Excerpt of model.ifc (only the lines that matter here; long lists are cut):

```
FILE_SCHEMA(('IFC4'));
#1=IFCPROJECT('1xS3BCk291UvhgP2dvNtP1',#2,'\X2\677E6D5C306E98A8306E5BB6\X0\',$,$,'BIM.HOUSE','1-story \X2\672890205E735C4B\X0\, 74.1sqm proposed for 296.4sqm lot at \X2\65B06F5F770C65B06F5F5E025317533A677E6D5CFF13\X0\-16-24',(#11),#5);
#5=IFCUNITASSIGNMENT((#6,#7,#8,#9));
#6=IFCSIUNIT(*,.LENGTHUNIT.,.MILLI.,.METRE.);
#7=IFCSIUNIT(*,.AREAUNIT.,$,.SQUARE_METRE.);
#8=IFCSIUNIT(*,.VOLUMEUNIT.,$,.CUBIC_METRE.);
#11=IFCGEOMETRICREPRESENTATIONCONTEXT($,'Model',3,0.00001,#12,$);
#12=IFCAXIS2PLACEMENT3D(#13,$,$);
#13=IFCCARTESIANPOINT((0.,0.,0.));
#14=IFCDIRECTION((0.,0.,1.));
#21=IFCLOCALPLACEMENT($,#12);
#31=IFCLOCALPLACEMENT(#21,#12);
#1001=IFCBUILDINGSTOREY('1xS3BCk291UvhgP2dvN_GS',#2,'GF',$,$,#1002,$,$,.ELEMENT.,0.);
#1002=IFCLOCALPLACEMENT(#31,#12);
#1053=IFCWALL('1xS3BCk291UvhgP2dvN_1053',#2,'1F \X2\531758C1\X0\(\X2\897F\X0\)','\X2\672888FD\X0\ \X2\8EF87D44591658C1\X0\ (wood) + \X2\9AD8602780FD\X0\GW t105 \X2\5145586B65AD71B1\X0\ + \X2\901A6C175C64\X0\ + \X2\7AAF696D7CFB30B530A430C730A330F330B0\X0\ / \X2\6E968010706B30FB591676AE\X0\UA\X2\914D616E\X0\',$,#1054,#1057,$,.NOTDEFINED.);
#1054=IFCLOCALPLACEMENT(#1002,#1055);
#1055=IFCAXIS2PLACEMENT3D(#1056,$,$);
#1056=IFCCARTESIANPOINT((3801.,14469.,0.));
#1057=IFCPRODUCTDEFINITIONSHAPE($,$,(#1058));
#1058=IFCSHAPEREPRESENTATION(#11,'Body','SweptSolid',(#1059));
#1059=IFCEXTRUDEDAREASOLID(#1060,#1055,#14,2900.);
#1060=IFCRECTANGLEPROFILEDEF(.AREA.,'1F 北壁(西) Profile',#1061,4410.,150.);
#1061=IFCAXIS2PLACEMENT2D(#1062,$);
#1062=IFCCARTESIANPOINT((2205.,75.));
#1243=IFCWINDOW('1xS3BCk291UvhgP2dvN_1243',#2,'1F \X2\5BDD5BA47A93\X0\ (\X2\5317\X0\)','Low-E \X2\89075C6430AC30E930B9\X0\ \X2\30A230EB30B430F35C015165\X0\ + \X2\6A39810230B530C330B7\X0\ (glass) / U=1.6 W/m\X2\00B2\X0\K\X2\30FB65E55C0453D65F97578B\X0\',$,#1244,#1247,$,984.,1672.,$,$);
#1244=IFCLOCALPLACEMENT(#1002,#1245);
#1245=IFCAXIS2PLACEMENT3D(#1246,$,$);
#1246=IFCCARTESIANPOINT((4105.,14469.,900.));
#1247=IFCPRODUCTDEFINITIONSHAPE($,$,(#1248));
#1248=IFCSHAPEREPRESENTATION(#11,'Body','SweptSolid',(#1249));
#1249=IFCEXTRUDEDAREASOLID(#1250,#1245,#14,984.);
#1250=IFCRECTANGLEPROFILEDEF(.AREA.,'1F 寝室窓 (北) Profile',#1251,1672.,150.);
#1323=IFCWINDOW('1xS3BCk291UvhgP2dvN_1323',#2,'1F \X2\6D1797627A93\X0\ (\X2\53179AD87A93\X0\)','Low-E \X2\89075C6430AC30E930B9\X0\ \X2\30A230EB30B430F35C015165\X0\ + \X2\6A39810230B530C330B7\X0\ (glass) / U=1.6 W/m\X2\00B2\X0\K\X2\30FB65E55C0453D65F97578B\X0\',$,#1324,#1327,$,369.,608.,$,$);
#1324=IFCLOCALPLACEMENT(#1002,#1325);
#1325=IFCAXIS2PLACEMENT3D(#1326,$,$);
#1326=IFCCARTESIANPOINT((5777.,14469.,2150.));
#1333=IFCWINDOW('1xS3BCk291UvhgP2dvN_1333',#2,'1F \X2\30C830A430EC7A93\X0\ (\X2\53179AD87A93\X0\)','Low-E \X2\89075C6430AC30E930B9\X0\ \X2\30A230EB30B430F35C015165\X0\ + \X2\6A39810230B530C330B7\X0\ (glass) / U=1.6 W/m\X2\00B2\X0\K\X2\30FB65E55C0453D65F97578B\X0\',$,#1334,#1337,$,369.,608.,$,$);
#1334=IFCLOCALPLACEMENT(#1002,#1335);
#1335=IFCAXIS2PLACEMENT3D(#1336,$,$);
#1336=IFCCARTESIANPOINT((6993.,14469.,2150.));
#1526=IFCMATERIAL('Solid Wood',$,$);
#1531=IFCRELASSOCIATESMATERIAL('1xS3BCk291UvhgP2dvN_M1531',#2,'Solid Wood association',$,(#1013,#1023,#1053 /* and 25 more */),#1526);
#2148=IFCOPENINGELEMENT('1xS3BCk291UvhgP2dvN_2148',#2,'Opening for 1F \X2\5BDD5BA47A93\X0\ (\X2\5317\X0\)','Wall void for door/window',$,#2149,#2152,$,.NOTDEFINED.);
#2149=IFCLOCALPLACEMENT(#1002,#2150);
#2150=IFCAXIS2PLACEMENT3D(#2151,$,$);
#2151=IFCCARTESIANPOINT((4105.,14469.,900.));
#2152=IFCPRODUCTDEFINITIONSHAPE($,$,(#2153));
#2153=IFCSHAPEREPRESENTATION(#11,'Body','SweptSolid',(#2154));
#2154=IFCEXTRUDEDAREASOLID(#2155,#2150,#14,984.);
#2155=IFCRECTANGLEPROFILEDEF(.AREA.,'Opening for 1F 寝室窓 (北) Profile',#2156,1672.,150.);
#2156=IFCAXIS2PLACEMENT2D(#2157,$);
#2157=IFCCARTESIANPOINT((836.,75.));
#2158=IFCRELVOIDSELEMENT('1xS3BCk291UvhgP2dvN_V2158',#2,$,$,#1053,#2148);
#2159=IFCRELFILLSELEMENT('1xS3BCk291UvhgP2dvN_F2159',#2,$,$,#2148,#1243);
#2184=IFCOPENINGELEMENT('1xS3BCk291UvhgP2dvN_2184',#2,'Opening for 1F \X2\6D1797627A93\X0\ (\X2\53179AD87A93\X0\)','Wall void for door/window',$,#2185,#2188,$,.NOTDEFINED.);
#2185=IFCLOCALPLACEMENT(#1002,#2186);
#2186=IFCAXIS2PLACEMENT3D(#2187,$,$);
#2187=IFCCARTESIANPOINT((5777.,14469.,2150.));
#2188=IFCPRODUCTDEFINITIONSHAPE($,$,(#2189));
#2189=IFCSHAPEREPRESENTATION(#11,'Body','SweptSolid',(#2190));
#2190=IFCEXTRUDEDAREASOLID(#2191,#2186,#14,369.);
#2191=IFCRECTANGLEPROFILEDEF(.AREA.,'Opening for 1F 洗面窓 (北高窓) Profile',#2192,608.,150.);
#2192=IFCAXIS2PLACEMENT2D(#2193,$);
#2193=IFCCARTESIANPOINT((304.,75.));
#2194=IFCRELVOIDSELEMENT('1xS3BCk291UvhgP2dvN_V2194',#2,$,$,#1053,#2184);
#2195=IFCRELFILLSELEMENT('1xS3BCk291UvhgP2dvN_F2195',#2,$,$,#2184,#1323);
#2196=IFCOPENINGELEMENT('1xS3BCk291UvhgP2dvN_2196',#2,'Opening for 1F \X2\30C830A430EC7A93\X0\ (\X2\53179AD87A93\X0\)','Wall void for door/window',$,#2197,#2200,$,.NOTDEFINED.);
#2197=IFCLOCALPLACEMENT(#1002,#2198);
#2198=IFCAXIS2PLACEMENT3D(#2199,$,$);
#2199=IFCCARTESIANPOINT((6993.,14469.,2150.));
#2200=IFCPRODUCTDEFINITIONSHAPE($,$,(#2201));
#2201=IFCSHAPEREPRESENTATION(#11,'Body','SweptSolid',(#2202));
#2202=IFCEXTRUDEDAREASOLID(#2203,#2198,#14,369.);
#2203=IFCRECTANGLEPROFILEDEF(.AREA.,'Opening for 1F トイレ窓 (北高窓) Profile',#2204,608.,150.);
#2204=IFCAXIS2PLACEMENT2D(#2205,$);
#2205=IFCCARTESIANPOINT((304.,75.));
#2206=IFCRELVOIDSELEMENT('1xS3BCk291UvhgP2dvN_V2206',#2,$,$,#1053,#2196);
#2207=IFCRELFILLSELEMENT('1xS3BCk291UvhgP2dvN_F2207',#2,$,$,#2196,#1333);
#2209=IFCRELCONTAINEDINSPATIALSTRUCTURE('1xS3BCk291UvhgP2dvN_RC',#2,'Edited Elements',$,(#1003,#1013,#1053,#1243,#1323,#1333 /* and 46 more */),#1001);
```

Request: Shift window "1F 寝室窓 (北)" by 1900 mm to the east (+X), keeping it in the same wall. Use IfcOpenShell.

```python
import ifcopenshell
import ifcopenshell.api.geometry
import ifcopenshell.util.placement
import ifcopenshell.util.unit

model = ifcopenshell.open("model.ifc")
unit_scale = ifcopenshell.util.unit.calculate_unit_scale(model)

window = model.by_id(1243)
opening = window.FillsVoids[0].RelatingOpeningElement
wall = opening.VoidsElements[0].RelatingBuildingElement

wall_matrix = ifcopenshell.util.placement.get_local_placement(wall.ObjectPlacement)
shift = wall_matrix[:3, 0] * 1.9 / unit_scale
before = ifcopenshell.util.placement.get_local_placement(window.ObjectPlacement)[:3, 3].copy()

# The window is not placed relative to its opening, so move both.
for product in (opening, window):
    matrix = ifcopenshell.util.placement.get_local_placement(product.ObjectPlacement)
    matrix[:3, 3] += shift
    ifcopenshell.api.geometry.edit_object_placement(model, product=product, matrix=matrix, is_si=False)

after = ifcopenshell.util.placement.get_local_placement(window.ObjectPlacement)[:3, 3]
print("window moved by", (after - before).round(3) + 0.0)

model.write("model_rev.ifc")
```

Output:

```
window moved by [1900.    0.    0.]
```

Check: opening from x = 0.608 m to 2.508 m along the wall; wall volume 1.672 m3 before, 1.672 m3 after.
